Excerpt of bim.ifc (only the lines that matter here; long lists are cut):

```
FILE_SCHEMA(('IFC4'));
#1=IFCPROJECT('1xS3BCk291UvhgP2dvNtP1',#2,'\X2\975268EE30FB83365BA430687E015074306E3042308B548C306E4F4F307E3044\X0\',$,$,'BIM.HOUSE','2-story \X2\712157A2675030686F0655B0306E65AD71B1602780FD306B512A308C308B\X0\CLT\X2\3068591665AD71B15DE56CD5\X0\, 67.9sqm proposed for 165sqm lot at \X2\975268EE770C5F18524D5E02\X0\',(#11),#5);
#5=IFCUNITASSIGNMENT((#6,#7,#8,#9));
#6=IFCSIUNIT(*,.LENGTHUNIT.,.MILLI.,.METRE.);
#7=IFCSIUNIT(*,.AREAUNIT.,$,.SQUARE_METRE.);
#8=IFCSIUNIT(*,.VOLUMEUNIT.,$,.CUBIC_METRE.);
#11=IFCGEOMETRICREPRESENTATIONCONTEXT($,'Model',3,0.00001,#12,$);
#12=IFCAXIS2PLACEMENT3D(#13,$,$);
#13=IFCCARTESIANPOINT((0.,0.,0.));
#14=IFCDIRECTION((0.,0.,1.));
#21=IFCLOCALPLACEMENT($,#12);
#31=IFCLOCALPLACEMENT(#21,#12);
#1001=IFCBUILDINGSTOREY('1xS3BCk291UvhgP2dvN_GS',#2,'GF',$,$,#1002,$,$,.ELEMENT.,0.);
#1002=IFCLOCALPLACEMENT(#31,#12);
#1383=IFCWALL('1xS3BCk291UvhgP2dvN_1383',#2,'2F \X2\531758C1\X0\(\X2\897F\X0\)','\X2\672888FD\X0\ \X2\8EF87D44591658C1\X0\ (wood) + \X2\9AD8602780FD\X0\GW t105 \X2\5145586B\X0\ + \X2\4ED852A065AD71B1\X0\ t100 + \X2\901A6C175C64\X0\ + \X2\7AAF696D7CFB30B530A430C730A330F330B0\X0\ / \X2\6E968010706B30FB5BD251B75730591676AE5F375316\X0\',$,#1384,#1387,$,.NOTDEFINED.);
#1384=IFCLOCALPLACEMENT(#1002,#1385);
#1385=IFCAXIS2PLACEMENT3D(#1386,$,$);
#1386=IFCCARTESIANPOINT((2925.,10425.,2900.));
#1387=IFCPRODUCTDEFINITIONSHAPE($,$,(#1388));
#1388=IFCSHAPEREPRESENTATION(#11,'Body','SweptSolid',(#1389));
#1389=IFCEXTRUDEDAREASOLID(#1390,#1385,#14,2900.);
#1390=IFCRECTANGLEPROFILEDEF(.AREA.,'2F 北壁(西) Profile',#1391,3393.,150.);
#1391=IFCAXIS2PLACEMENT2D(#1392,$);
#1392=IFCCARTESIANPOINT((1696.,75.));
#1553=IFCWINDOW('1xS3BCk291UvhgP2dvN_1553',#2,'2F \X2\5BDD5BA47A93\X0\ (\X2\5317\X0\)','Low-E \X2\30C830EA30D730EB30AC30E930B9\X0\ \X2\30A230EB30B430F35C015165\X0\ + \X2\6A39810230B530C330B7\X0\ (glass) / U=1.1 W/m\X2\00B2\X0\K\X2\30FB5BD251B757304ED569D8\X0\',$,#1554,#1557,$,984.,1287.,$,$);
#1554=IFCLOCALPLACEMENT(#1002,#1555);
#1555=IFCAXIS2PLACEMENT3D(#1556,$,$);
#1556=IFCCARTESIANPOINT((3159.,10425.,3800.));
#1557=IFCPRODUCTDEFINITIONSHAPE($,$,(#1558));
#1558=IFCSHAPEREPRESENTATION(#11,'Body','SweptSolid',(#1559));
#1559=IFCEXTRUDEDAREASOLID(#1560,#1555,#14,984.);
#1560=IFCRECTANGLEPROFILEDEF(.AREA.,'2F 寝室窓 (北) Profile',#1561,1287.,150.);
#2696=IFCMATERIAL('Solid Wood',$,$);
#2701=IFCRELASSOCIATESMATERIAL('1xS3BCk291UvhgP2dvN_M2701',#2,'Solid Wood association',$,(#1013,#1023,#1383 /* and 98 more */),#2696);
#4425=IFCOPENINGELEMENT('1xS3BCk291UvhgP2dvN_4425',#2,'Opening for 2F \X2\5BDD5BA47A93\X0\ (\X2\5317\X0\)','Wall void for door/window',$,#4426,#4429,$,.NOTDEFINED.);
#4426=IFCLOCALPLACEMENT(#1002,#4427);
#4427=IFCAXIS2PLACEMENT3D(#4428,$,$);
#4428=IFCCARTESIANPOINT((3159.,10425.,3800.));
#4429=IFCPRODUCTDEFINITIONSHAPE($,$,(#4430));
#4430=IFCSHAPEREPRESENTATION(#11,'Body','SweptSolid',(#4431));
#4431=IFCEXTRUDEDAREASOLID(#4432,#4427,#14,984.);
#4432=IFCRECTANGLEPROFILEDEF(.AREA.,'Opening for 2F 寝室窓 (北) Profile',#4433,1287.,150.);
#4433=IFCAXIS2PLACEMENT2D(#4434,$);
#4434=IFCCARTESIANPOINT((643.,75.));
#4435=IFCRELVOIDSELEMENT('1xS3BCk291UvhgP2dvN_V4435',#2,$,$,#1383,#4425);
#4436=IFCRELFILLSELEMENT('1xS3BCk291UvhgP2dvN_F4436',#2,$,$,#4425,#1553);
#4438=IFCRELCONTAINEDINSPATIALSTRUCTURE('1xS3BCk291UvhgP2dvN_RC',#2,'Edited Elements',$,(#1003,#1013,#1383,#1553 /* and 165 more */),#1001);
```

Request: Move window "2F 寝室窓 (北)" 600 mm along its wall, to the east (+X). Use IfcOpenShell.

```python
import ifcopenshell
import ifcopenshell.api.geometry
import ifcopenshell.util.placement

model = ifcopenshell.open("bim.ifc")

window = model.by_guid("1xS3BCk291UvhgP2dvN_1553")
opening = window.FillsVoids[0].RelatingOpeningElement
wall = opening.VoidsElements[0].RelatingBuildingElement

wall_matrix = ifcopenshell.util.placement.get_local_placement(wall.ObjectPlacement)
shift = wall_matrix[:3, 0] * 600.0
before = ifcopenshell.util.placement.get_local_placement(window.ObjectPlacement)[:3, 3].copy()

# The window is not placed relative to its opening, so move both.
for product in (opening, window):
    matrix = ifcopenshell.util.placement.get_local_placement(product.ObjectPlacement)
    matrix[:3, 3] += shift
    ifcopenshell.api.geometry.edit_object_placement(model, product=product, matrix=matrix, is_si=False)

after = ifcopenshell.util.placement.get_local_placement(window.ObjectPlacement)[:3, 3]
print("window moved by", (after - before).round(3) + 0.0)

model.write("bim_rev.ifc")
```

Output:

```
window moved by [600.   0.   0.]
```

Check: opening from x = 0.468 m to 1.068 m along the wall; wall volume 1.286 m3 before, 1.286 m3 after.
